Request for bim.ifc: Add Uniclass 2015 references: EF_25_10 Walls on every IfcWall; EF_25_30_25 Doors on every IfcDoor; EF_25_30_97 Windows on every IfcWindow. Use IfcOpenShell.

First a look at what the model holds.

```python
import ifcopenshell

model = ifcopenshell.open("bim.ifc")
print(model.schema)
print("classifications:", [c.Name for c in model.by_type("IfcClassification")])
for ifc_class in ("IfcDoor", "IfcRoof", "IfcStair", "IfcWall", "IfcWindow"):
    print(ifc_class, len(model.by_type(ifc_class)))
```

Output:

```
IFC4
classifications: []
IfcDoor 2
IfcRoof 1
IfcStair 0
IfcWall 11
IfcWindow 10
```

```python
import ifcopenshell
import ifcopenshell.api.classification

model = ifcopenshell.open("bim.ifc")

system = ifcopenshell.api.classification.add_classification(model, classification="Uniclass 2015")

codes = {
    "IfcWall": ("EF_25_10", "Walls"),
    "IfcDoor": ("EF_25_30_25", "Doors"),
    "IfcWindow": ("EF_25_30_97", "Windows"),
}
for ifc_class, (code, name) in codes.items():
    products = model.by_type(ifc_class)
    ifcopenshell.api.classification.add_reference(
        model, products=products, classification=system, identification=code, name=name
    )
    print(code, len(products))

model.write("bim-out.ifc")
```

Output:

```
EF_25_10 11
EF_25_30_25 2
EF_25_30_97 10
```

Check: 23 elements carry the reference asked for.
